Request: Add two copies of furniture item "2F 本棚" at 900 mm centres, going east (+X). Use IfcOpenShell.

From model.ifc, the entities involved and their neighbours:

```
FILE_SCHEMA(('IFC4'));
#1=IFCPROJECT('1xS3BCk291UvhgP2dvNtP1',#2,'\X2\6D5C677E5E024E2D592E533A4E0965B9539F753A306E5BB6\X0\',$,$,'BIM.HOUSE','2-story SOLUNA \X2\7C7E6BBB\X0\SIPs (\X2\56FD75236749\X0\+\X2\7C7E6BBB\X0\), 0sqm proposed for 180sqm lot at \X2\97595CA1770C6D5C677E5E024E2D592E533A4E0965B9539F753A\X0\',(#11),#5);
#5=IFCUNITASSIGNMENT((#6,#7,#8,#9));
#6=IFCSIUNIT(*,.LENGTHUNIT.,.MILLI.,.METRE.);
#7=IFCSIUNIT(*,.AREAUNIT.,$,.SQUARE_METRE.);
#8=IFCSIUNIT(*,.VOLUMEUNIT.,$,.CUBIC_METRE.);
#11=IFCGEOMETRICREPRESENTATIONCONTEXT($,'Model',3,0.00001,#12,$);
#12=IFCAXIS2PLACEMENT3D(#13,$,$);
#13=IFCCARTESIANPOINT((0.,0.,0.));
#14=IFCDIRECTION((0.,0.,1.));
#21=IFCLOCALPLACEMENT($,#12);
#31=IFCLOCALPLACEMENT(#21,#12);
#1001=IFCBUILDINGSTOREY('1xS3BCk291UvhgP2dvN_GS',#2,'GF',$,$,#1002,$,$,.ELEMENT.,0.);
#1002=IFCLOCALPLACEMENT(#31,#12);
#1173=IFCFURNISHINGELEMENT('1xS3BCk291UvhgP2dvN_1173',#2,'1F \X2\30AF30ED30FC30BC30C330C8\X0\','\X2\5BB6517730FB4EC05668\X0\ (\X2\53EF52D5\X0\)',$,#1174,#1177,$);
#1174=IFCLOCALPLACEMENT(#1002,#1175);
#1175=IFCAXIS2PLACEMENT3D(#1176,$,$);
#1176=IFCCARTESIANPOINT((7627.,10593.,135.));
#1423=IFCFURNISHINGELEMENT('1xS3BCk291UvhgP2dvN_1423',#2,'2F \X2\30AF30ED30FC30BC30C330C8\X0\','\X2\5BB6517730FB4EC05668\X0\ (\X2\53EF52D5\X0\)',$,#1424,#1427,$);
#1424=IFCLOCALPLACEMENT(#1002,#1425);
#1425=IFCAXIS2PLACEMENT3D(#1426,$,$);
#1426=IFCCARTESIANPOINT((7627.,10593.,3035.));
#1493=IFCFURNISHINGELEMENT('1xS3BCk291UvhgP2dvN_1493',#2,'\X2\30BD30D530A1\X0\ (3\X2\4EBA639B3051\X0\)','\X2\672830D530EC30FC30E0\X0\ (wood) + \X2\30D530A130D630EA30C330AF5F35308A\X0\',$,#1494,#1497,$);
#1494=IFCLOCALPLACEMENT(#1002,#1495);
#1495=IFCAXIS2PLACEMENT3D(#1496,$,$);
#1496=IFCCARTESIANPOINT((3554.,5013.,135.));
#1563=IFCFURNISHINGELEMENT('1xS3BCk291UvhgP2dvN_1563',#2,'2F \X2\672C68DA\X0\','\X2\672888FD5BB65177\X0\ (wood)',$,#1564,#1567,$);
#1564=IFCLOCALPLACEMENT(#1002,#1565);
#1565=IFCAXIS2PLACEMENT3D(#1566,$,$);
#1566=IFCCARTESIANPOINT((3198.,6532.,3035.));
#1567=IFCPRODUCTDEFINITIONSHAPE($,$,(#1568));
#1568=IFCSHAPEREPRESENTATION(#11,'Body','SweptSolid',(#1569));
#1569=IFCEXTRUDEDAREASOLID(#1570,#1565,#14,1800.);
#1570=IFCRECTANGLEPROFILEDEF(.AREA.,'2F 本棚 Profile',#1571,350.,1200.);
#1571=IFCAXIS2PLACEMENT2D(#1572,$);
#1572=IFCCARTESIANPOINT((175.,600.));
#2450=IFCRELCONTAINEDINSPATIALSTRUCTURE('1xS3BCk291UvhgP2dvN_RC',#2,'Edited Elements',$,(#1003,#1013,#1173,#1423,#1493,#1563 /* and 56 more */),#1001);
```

```python
import numpy as np
import ifcopenshell
import ifcopenshell.api.geometry
import ifcopenshell.api.root
import ifcopenshell.util.element
import ifcopenshell.util.placement

model = ifcopenshell.open("model.ifc")


def reuse_history(source, copy):
    """copy_class also copies each property set's owner history, people and application; keep the originals."""
    for rel in copy.IsDefinedBy:
        if rel.is_a("IfcRelDefinesByProperties") and (history := rel.RelatingPropertyDefinition.OwnerHistory):
            rel.RelatingPropertyDefinition.OwnerHistory = source.OwnerHistory
            ifcopenshell.util.element.remove_deep2(model, history)


source = model.by_id(1563)
base = ifcopenshell.util.placement.get_local_placement(source.ObjectPlacement)
step = np.array([1.0, 0.0, 0.0]) * 900.0

for i in range(1, 3):
    copy = ifcopenshell.api.root.copy_class(model, product=source)
    copy.Representation = ifcopenshell.util.element.copy_deep(
        model, source.Representation, exclude=["IfcGeometricRepresentationContext", "IfcRepresentationMap"]
    )
    reuse_history(source, copy)
    matrix = base.copy()
    matrix[:3, 3] += i * step
    print("added at", matrix[:3, 3].round(3) + 0.0)
    ifcopenshell.api.geometry.edit_object_placement(model, product=copy, matrix=matrix, is_si=False)

model.write("model_updated.ifc")
```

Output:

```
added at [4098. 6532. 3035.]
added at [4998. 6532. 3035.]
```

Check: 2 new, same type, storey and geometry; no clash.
